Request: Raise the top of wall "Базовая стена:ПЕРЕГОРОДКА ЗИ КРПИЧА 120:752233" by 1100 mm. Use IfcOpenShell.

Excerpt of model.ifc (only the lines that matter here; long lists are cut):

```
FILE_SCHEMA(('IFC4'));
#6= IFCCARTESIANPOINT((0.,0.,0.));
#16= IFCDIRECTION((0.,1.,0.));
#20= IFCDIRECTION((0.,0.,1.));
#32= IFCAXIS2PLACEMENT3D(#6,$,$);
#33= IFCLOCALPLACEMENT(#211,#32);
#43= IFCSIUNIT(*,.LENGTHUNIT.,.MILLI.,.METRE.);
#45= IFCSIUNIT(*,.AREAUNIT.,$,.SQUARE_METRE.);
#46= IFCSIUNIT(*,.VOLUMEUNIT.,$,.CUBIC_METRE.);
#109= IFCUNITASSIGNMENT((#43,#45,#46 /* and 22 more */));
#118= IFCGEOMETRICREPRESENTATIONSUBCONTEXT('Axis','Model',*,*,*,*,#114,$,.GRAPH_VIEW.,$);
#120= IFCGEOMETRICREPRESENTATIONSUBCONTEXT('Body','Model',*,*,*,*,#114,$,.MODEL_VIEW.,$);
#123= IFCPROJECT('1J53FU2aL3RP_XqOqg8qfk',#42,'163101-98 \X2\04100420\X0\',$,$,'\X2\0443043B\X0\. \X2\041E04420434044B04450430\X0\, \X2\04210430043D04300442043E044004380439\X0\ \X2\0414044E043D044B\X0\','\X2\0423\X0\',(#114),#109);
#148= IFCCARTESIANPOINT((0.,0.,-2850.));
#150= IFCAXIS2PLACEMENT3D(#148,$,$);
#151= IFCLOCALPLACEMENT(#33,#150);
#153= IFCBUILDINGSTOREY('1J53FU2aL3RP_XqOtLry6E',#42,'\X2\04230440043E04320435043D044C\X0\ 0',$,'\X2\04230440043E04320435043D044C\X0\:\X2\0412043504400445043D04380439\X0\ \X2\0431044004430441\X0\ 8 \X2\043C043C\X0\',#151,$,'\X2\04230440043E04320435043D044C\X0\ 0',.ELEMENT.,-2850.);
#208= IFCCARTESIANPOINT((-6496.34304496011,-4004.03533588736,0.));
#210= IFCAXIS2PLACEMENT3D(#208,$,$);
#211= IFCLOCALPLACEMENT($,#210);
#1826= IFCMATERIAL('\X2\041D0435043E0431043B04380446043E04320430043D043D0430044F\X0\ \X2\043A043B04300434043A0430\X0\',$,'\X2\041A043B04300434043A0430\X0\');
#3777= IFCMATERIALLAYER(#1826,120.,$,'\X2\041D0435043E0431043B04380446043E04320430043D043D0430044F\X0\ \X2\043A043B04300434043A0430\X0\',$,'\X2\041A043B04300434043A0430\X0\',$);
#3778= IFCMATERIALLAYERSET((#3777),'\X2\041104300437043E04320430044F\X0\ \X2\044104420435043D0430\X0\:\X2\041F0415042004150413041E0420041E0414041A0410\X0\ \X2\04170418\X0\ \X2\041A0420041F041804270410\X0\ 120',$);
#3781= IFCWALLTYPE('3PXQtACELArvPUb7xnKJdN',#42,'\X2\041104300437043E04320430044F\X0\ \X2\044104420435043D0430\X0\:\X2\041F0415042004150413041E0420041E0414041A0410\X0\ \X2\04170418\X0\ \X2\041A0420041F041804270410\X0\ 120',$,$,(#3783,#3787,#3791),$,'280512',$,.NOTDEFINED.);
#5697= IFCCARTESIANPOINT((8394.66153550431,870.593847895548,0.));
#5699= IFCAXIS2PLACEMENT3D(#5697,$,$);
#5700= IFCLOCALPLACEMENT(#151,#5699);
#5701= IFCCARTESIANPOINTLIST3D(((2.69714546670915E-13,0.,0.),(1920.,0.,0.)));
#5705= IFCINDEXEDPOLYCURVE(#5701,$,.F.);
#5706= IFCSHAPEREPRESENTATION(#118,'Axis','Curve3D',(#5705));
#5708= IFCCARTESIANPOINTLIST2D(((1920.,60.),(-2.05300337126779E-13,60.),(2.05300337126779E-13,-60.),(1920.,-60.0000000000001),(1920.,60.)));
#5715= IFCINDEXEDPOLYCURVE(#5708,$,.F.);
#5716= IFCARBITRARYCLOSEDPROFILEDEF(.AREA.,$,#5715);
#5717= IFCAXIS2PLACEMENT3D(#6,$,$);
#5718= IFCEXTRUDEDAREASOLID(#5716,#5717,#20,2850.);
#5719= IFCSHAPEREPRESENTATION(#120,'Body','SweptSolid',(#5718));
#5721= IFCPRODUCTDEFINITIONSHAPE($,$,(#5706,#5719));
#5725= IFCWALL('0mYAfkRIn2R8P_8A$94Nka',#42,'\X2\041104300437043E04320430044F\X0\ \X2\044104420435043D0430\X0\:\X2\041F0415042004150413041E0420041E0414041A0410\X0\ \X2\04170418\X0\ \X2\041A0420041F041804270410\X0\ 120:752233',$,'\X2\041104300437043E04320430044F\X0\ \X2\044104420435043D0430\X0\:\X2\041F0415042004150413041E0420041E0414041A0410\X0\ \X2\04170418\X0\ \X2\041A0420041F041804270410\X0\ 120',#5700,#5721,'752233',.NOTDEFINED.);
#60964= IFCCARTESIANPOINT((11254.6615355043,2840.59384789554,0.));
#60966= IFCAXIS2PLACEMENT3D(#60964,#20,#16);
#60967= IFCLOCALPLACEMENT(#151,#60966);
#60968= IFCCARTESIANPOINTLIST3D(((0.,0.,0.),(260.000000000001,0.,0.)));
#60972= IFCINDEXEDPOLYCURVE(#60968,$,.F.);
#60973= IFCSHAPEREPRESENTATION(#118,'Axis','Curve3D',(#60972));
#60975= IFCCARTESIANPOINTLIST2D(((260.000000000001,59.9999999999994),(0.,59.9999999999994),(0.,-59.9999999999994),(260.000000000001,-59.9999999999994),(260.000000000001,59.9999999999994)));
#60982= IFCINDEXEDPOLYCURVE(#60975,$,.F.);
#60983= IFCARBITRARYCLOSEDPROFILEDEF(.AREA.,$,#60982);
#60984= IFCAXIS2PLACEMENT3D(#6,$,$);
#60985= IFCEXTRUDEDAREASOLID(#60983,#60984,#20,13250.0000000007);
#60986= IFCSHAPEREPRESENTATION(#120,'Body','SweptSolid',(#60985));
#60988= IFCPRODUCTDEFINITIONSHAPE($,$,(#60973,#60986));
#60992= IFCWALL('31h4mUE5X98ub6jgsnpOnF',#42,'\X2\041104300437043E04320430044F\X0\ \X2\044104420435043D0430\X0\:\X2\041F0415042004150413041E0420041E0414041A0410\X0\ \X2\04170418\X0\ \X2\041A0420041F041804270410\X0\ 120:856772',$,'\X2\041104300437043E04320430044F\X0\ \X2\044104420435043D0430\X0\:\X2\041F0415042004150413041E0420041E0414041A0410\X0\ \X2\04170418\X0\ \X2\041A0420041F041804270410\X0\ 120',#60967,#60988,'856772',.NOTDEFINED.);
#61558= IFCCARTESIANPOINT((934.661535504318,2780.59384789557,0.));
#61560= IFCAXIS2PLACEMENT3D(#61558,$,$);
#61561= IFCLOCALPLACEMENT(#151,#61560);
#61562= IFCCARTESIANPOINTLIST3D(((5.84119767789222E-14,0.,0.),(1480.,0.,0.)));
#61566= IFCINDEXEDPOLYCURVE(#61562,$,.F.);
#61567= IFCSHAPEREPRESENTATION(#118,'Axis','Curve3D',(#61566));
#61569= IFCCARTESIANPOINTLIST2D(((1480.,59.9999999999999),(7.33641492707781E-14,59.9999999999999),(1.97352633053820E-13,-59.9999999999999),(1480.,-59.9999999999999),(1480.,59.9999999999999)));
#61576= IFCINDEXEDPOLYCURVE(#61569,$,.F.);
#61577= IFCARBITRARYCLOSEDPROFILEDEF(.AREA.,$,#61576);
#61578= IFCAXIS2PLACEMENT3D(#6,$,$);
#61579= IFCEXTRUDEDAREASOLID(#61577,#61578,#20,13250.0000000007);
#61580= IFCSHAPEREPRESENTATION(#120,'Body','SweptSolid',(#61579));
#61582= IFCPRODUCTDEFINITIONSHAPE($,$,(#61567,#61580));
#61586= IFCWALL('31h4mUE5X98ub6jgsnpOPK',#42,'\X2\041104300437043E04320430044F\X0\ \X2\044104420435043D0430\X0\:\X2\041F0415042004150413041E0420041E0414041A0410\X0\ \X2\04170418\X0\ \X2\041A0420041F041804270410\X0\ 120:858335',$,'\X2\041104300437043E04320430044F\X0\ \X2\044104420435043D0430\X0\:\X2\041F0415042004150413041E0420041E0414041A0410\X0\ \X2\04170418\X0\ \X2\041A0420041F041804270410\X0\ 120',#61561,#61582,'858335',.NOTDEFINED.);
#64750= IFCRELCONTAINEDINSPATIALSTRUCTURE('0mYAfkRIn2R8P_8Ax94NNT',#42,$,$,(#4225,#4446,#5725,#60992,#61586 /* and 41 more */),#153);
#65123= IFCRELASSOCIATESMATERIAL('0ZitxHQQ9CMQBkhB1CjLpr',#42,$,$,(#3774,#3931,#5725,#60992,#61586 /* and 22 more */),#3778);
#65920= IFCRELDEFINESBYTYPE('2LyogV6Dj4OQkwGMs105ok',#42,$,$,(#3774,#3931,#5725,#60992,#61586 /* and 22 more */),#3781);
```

```python
import ifcopenshell
import ifcopenshell.geom
import ifcopenshell.util.representation
import ifcopenshell.util.shape

model = ifcopenshell.open("model.ifc")
settings = ifcopenshell.geom.settings()


def volume(element):
    """Net volume in cubic metres, openings subtracted."""
    shape = ifcopenshell.geom.create_shape(settings, element)
    return ifcopenshell.util.shape.get_volume(shape.geometry)


wall = model.by_guid("0mYAfkRIn2R8P_8A$94Nka")
before = volume(wall)

body = ifcopenshell.util.representation.get_representation(wall, "Model", "Body")
solid = body.Items[0]
old_height = solid.Depth
solid.Depth += 1100.0
after = volume(wall)

print(f"height {old_height:g} -> {solid.Depth:g}, volume {before:.3f} -> {after:.3f} m3")

model.write("model-out.ifc")
```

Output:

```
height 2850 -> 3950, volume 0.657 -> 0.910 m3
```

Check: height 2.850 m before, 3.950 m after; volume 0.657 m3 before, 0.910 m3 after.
